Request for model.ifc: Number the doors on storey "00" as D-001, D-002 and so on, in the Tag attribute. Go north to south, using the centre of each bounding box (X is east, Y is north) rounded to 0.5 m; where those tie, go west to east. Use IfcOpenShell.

First a look at what the model holds.

```python
import ifcopenshell
import ifcopenshell.util.element
import ifcopenshell.util.placement

model = ifcopenshell.open("model.ifc")
print(model.schema)
storey = next(s for s in model.by_type("IfcBuildingStorey") if s.Name == "00")
doors = [e for e in ifcopenshell.util.element.get_decomposition(storey) if e.is_a("IfcDoor")]
for e in sorted(doors, key=lambda e: e.id()):
    origin = ifcopenshell.util.placement.get_local_placement(e.ObjectPlacement)[:3, 3]
    print(e.id(), e.Tag, e.Name, origin.round(2) + 0.0, sep=" | ")
```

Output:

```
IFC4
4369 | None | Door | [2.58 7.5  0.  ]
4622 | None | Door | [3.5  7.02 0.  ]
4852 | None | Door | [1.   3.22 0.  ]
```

```python
import ifcopenshell
import ifcopenshell.geom
import ifcopenshell.util.element
import ifcopenshell.util.shape

model = ifcopenshell.open("model.ifc")
settings = ifcopenshell.geom.settings()
settings.set("use-world-coords", True)


def centre(element):
    shape = ifcopenshell.geom.create_shape(settings, element)
    return ifcopenshell.util.shape.get_bbox_centroid(shape.geometry)


storey = next(s for s in model.by_type("IfcBuildingStorey") if s.Name == "00")
doors = [e for e in ifcopenshell.util.element.get_decomposition(storey) if e.is_a("IfcDoor")]

# Insertion points can sit at a corner or the storey origin, so sort by the geometry (in metres).
centres = {e: centre(e) for e in doors}
doors.sort(key=lambda e: (-round(centres[e][1] / 0.5), centres[e][0]))

for i, e in enumerate(doors, start=1):
    number = f"D-0{i:02d}"
    e.Tag = number
    print(e.id(), number)

model.write("model_v2.ifc")
```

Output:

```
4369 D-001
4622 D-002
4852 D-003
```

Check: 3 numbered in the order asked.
